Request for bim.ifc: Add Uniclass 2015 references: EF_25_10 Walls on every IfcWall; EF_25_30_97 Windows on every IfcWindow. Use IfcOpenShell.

First a look at what the model holds.

```python
import ifcopenshell

model = ifcopenshell.open("bim.ifc")
print(model.schema)
print("classifications:", [c.Name for c in model.by_type("IfcClassification")])
for ifc_class in ("IfcDoor", "IfcRoof", "IfcStair", "IfcWall", "IfcWindow"):
    print(ifc_class, len(model.by_type(ifc_class)))
```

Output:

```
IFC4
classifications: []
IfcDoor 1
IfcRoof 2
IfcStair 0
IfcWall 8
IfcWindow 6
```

```python
import ifcopenshell
import ifcopenshell.api.classification

model = ifcopenshell.open("bim.ifc")

system = ifcopenshell.api.classification.add_classification(model, classification="Uniclass 2015")

codes = {
    "IfcWall": ("EF_25_10", "Walls"),
    "IfcWindow": ("EF_25_30_97", "Windows"),
}
for ifc_class, (code, name) in codes.items():
    products = model.by_type(ifc_class)
    ifcopenshell.api.classification.add_reference(
        model, products=products, classification=system, identification=code, name=name
    )
    print(code, len(products))

model.write("bim_edited.ifc")
```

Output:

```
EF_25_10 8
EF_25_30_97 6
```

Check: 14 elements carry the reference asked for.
